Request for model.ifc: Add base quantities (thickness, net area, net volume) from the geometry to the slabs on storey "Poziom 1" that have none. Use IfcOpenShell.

First a look at what the model holds.

```python
import ifcopenshell
import ifcopenshell.util.element
import ifcopenshell.util.unit

model = ifcopenshell.open("model.ifc")
print(model.schema)
for unit_type in ("LENGTHUNIT", "AREAUNIT", "VOLUMEUNIT"):
    print(unit_type, ifcopenshell.util.unit.calculate_unit_scale(model, unit_type))
storey = next(s for s in model.by_type("IfcBuildingStorey") if s.Name == "Poziom 1")
slabs = [e for e in ifcopenshell.util.element.get_decomposition(storey) if e.is_a("IfcSlab")]
for e in sorted(slabs, key=lambda e: e.id()):
    print(e.id(), e.is_a(), e.Name, list(ifcopenshell.util.element.get_psets(e, qtos_only=True)), sep=" | ")
```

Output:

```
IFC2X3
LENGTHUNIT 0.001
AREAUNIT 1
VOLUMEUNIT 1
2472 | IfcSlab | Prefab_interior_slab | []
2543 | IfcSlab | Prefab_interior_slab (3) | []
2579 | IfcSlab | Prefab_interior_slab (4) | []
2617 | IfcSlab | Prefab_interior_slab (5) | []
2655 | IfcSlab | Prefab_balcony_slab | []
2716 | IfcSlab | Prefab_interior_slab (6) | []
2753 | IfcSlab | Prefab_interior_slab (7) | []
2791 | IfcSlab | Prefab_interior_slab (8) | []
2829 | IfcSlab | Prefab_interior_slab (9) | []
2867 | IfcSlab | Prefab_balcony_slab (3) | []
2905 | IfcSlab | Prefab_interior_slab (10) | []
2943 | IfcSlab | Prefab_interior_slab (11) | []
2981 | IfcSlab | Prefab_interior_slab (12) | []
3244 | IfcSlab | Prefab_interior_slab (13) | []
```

```python
import ifcopenshell
import ifcopenshell.api.pset
import ifcopenshell.geom
import ifcopenshell.util.element
import ifcopenshell.util.shape
import ifcopenshell.util.unit

model = ifcopenshell.open("model.ifc")
unit_scale = ifcopenshell.util.unit.calculate_unit_scale(model)
area_scale = ifcopenshell.util.unit.calculate_unit_scale(model, "AREAUNIT")
volume_scale = ifcopenshell.util.unit.calculate_unit_scale(model, "VOLUMEUNIT")
settings = ifcopenshell.geom.settings()

storey = next(s for s in model.by_type("IfcBuildingStorey") if s.Name == "Poziom 1")
slabs = [e for e in ifcopenshell.util.element.get_decomposition(storey) if e.is_a("IfcSlab")]

for e in sorted(slabs, key=lambda e: e.id()):
    if ifcopenshell.util.element.get_psets(e, qtos_only=True, should_inherit=False):
        continue
    # Geometry comes back in metres, in the element's own axes.
    shape = ifcopenshell.geom.create_shape(settings, e)
    values = {
        "Width": ifcopenshell.util.shape.get_z(shape.geometry) / unit_scale,
        "NetArea": ifcopenshell.util.shape.get_footprint_area(shape.geometry) / area_scale,
        "NetVolume": ifcopenshell.util.shape.get_volume(shape.geometry) / volume_scale,
    }
    qto = ifcopenshell.api.pset.add_qto(model, product=e, name="BaseQuantities")
    ifcopenshell.api.pset.edit_qto(model, qto=qto, properties=values)
    print(e.id(), {k: round(v, 3) for k, v in values.items()})

model.write("model_v2.ifc")
```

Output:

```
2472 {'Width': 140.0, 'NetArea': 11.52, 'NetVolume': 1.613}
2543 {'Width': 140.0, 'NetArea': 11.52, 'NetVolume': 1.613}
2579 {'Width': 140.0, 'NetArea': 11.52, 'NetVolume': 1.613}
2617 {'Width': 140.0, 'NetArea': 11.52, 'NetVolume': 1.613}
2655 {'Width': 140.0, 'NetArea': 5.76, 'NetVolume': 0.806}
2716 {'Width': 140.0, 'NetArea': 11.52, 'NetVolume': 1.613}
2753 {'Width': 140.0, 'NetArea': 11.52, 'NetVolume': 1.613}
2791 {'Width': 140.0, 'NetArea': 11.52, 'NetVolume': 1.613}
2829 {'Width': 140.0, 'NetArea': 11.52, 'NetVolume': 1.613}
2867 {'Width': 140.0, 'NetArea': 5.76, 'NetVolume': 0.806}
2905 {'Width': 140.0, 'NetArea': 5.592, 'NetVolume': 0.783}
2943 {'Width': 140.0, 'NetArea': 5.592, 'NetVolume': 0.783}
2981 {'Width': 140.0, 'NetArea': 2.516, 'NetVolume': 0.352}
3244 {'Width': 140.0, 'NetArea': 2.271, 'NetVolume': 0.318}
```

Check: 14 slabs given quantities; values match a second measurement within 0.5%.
